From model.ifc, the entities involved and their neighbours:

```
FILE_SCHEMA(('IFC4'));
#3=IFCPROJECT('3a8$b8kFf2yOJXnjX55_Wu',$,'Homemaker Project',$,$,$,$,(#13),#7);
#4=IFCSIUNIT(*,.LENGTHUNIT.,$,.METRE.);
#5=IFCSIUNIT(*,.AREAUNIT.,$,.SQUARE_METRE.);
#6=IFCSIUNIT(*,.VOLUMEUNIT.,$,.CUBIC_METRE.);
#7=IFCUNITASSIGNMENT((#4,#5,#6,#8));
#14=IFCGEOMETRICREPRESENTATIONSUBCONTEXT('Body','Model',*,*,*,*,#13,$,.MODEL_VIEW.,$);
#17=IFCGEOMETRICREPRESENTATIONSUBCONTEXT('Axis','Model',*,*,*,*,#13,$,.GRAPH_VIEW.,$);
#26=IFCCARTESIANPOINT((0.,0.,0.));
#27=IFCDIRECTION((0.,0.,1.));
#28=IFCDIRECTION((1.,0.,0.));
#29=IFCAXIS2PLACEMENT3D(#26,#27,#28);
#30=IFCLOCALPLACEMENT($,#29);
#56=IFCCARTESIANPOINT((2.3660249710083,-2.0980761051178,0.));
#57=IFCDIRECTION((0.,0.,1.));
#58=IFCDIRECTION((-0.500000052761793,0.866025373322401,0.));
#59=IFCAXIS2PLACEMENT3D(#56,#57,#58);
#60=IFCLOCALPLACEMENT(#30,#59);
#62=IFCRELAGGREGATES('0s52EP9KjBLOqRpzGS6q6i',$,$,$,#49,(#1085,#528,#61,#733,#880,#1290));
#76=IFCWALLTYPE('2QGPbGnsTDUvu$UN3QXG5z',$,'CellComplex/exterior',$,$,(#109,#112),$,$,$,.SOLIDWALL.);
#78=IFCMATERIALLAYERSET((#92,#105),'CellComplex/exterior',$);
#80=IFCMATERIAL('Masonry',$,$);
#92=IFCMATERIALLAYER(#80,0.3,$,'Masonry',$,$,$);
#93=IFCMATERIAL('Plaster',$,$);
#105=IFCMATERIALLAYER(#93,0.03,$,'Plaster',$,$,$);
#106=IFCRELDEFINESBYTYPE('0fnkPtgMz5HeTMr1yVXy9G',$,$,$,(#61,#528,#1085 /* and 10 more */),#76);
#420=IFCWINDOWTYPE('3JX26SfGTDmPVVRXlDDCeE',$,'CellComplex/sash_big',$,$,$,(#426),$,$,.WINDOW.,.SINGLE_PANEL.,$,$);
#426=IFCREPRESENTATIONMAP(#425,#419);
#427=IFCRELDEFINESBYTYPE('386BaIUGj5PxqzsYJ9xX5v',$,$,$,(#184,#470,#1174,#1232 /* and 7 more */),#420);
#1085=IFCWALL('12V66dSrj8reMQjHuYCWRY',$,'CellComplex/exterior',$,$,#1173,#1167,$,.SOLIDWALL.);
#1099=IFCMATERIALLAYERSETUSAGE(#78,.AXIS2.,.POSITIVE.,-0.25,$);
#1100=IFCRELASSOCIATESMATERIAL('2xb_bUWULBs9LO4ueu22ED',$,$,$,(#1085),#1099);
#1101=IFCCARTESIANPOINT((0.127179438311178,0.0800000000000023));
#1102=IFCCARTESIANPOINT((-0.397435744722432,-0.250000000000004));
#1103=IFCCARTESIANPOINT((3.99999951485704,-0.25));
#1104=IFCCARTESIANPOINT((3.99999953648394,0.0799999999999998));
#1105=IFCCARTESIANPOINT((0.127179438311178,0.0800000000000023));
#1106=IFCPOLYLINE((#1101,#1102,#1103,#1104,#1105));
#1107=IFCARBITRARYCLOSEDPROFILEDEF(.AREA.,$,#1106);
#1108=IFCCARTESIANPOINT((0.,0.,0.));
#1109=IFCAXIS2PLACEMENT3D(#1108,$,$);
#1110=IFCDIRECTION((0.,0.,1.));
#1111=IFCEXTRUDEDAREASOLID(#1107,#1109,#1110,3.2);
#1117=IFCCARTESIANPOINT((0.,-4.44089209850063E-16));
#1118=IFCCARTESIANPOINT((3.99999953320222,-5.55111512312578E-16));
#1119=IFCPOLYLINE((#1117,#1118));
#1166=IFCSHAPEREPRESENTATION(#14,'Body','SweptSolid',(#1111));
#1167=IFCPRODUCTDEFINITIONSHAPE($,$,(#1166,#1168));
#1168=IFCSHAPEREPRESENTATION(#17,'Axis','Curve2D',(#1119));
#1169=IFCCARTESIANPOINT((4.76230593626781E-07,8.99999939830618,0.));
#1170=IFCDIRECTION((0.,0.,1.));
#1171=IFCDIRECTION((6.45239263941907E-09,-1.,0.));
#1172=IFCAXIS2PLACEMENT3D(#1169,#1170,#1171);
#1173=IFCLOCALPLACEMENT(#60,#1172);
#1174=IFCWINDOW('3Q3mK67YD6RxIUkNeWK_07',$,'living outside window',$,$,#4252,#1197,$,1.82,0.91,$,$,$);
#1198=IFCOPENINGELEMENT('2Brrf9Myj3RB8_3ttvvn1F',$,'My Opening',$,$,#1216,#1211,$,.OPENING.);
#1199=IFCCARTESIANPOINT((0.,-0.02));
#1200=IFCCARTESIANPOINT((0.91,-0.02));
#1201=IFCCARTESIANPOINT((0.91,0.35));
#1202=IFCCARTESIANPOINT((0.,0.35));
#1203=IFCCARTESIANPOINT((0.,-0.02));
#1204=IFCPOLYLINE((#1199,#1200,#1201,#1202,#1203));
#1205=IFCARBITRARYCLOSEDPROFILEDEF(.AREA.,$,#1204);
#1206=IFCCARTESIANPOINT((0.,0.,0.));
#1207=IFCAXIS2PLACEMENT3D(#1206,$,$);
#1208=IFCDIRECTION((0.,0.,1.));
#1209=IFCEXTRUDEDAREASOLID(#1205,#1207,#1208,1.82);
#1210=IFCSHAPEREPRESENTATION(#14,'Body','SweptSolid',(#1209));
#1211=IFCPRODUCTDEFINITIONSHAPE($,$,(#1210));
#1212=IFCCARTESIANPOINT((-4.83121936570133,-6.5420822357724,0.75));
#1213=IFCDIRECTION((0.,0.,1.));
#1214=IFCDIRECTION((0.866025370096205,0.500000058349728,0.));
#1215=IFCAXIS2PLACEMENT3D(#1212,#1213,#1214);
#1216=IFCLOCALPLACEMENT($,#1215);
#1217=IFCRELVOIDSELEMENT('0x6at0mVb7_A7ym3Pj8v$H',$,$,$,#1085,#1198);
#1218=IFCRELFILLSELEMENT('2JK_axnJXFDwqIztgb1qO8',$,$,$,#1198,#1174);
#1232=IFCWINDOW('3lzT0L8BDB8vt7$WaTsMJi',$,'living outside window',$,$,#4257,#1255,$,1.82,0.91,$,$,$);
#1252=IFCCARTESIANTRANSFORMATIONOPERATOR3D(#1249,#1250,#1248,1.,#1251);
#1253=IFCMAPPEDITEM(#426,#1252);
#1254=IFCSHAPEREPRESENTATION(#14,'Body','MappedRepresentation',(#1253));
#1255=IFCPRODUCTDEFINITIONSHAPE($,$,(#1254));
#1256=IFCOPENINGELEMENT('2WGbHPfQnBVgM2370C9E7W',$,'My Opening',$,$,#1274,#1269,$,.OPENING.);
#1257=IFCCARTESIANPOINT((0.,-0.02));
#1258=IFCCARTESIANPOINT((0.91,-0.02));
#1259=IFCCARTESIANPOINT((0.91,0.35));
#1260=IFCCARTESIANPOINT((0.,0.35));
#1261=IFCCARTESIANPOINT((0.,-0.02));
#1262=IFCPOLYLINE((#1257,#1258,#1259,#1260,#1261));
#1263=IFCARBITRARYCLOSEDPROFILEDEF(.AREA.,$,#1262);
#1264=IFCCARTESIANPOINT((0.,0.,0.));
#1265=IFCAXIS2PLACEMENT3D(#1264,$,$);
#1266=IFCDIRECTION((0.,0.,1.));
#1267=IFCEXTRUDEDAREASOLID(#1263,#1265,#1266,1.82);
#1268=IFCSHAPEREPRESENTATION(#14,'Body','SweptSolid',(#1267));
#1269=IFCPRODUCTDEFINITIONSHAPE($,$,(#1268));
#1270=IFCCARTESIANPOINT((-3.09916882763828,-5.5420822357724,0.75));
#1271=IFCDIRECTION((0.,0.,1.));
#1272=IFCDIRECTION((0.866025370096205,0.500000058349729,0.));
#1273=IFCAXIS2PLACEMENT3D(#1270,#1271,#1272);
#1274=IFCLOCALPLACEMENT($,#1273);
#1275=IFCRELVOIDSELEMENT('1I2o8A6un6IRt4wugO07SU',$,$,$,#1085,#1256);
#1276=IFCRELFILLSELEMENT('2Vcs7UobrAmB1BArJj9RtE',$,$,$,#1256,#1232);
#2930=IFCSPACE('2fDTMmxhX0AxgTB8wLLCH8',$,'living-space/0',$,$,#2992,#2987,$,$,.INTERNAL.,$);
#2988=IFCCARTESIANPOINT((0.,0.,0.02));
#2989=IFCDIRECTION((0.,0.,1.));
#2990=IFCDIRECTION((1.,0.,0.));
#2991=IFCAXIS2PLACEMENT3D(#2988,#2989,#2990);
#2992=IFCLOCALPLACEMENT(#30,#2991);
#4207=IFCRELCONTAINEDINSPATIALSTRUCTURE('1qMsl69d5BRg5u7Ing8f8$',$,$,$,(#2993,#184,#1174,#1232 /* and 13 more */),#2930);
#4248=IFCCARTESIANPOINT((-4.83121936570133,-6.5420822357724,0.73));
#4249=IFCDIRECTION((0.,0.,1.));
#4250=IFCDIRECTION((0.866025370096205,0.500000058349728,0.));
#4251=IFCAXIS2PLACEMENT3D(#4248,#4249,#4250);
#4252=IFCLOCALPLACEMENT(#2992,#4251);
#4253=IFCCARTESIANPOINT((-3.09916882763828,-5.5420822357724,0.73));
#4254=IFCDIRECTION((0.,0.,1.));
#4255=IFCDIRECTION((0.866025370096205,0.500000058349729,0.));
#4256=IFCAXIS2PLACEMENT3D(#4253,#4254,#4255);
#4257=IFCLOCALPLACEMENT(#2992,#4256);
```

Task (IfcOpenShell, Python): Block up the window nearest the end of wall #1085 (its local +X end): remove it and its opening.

```python
import ifcopenshell
import ifcopenshell.api.feature
import ifcopenshell.api.root
import ifcopenshell.geom
import ifcopenshell.util.shape

model = ifcopenshell.open("model.ifc")
settings = ifcopenshell.geom.settings()


def volume(element):
    """Net volume in cubic metres, openings subtracted."""
    shape = ifcopenshell.geom.create_shape(settings, element)
    return ifcopenshell.util.shape.get_volume(shape.geometry)


window = model.by_guid("3lzT0L8BDB8vt7$WaTsMJi")
opening = window.FillsVoids[0].RelatingOpeningElement
wall = opening.VoidsElements[0].RelatingBuildingElement
before = volume(wall)

ifcopenshell.api.root.remove_product(model, product=window)
ifcopenshell.api.feature.remove_feature(model, feature=opening)

after = volume(wall)

print(f"wall volume {before:.3f} -> {after:.3f} m3")

model.write("model-out.ifc")
```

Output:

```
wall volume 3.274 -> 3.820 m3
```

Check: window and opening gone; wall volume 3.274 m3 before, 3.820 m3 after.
